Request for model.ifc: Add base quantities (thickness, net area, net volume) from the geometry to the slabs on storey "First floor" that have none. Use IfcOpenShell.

First a look at what the model holds.

```python
import ifcopenshell
import ifcopenshell.util.element
import ifcopenshell.util.unit

model = ifcopenshell.open("model.ifc")
print(model.schema)
for unit_type in ("LENGTHUNIT", "AREAUNIT", "VOLUMEUNIT"):
    print(unit_type, ifcopenshell.util.unit.calculate_unit_scale(model, unit_type))
storey = next(s for s in model.by_type("IfcBuildingStorey") if s.Name == "First floor")
slabs = [e for e in ifcopenshell.util.element.get_decomposition(storey) if e.is_a("IfcSlab")]
for e in sorted(slabs, key=lambda e: e.id()):
    print(e.id(), e.is_a(), e.Name, list(ifcopenshell.util.element.get_psets(e, qtos_only=True)), sep=" | ")
```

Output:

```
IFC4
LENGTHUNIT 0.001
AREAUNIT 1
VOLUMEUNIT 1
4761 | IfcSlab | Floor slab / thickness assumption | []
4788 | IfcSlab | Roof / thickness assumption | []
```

```python
import ifcopenshell
import ifcopenshell.api.pset
import ifcopenshell.geom
import ifcopenshell.util.element
import ifcopenshell.util.shape
import ifcopenshell.util.unit

model = ifcopenshell.open("model.ifc")
unit_scale = ifcopenshell.util.unit.calculate_unit_scale(model)
area_scale = ifcopenshell.util.unit.calculate_unit_scale(model, "AREAUNIT")
volume_scale = ifcopenshell.util.unit.calculate_unit_scale(model, "VOLUMEUNIT")
settings = ifcopenshell.geom.settings()

storey = next(s for s in model.by_type("IfcBuildingStorey") if s.Name == "First floor")
slabs = [e for e in ifcopenshell.util.element.get_decomposition(storey) if e.is_a("IfcSlab")]

for e in sorted(slabs, key=lambda e: e.id()):
    if ifcopenshell.util.element.get_psets(e, qtos_only=True, should_inherit=False):
        continue
    # Geometry comes back in metres, in the element's own axes.
    shape = ifcopenshell.geom.create_shape(settings, e)
    values = {
        "Width": ifcopenshell.util.shape.get_z(shape.geometry) / unit_scale,
        "NetArea": ifcopenshell.util.shape.get_footprint_area(shape.geometry) / area_scale,
        "NetVolume": ifcopenshell.util.shape.get_volume(shape.geometry) / volume_scale,
    }
    qto = ifcopenshell.api.pset.add_qto(model, product=e, name="Qto_SlabBaseQuantities")
    ifcopenshell.api.pset.edit_qto(model, qto=qto, properties=values)
    print(e.id(), {k: round(v, 3) for k, v in values.items()})

model.write("model-out.ifc")
```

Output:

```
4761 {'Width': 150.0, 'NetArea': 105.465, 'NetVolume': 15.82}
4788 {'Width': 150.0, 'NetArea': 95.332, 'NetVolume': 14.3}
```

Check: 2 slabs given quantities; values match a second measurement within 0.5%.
